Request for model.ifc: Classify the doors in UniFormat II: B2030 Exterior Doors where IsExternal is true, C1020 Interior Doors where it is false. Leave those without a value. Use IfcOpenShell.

First a look at what the model holds.

```python
import ifcopenshell
import ifcopenshell.util.element

model = ifcopenshell.open("model.ifc")
print(model.schema)
print("classifications:", [c.Name for c in model.by_type("IfcClassification")])
values = [ifcopenshell.util.element.get_pset(e, "Pset_DoorCommon", "IsExternal") for e in model.by_type("IfcDoor")]
for value in (True, False, None):
    print("IsExternal", value, values.count(value))
```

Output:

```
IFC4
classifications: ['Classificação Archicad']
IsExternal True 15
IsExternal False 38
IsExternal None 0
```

```python
import ifcopenshell
import ifcopenshell.api.classification
import ifcopenshell.util.element

model = ifcopenshell.open("model.ifc")

system = ifcopenshell.api.classification.add_classification(model, classification="UniFormat II")

doors = model.by_type("IfcDoor")
external = {e: ifcopenshell.util.element.get_pset(e, "Pset_DoorCommon", "IsExternal") for e in doors}
for flag, code, name in ((True, "B2030", "Exterior Doors"), (False, "C1020", "Interior Doors")):
    products = [e for e in doors if external[e] is flag]
    ifcopenshell.api.classification.add_reference(
        model, products=products, classification=system, identification=code, name=name
    )
    print(code, len(products))

model.write("model_edited.ifc")
```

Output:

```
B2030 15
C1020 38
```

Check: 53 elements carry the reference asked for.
